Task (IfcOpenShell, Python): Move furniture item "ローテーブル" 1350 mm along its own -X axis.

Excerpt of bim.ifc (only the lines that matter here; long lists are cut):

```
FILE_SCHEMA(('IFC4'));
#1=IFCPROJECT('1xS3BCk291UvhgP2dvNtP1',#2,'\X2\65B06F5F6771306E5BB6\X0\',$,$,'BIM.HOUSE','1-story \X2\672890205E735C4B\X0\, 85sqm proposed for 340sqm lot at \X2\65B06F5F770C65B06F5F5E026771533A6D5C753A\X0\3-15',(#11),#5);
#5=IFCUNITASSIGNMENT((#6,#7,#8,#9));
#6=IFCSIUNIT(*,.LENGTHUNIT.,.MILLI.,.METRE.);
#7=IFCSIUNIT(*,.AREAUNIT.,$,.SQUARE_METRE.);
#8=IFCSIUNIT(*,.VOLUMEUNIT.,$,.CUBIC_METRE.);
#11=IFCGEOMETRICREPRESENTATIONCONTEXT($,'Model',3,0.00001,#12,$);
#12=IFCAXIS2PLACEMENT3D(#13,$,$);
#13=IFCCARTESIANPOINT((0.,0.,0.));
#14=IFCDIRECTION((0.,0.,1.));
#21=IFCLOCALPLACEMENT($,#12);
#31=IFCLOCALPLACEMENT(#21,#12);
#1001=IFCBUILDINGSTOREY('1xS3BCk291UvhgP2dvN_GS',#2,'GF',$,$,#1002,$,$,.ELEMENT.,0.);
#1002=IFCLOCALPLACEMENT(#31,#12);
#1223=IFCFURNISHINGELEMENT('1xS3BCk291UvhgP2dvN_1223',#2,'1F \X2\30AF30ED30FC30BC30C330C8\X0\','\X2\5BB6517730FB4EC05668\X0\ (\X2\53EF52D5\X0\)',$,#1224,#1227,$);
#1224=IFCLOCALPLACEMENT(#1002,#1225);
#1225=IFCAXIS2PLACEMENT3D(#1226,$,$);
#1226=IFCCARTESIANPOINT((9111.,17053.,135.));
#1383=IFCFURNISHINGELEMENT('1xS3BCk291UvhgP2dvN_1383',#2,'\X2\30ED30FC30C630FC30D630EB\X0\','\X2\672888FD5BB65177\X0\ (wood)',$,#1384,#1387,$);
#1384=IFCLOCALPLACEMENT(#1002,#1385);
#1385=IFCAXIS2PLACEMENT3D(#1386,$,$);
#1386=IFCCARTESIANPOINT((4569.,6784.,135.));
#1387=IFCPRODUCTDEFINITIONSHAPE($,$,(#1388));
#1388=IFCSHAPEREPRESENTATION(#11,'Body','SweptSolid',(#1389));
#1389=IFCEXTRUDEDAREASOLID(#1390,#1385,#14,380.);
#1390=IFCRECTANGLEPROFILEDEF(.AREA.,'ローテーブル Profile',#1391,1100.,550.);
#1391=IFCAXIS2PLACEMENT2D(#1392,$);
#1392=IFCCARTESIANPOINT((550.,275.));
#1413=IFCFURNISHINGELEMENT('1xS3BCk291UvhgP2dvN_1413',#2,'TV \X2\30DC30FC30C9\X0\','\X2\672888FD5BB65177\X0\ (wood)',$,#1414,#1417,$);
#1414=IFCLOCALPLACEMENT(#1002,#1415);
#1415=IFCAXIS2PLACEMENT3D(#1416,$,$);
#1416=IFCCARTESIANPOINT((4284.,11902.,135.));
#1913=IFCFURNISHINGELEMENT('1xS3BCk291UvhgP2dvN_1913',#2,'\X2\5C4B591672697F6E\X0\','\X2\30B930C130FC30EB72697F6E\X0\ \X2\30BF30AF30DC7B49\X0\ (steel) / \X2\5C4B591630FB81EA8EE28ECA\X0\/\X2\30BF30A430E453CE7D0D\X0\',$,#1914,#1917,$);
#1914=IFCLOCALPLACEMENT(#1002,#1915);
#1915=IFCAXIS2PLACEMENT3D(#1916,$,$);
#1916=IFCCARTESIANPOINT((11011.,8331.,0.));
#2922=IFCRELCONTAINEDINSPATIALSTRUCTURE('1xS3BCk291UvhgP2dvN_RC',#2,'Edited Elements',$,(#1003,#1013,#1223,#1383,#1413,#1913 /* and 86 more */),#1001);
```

```python
import ifcopenshell
import ifcopenshell.api.geometry
import ifcopenshell.util.placement
import ifcopenshell.util.unit

model = ifcopenshell.open("bim.ifc")
unit_scale = ifcopenshell.util.unit.calculate_unit_scale(model)

item = model.by_id(1383)
matrix = ifcopenshell.util.placement.get_local_placement(item.ObjectPlacement)
matrix[:3, 3] -= matrix[:3, 0] * 1.35 / unit_scale
ifcopenshell.api.geometry.edit_object_placement(model, product=item, matrix=matrix, is_si=False)

print(ifcopenshell.util.placement.get_local_placement(item.ObjectPlacement).round(3) + 0.0)

model.write("bim_updated.ifc")
```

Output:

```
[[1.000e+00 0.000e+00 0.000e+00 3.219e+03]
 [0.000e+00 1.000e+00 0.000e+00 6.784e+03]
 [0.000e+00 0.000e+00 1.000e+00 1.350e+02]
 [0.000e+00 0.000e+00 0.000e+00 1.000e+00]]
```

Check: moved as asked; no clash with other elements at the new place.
